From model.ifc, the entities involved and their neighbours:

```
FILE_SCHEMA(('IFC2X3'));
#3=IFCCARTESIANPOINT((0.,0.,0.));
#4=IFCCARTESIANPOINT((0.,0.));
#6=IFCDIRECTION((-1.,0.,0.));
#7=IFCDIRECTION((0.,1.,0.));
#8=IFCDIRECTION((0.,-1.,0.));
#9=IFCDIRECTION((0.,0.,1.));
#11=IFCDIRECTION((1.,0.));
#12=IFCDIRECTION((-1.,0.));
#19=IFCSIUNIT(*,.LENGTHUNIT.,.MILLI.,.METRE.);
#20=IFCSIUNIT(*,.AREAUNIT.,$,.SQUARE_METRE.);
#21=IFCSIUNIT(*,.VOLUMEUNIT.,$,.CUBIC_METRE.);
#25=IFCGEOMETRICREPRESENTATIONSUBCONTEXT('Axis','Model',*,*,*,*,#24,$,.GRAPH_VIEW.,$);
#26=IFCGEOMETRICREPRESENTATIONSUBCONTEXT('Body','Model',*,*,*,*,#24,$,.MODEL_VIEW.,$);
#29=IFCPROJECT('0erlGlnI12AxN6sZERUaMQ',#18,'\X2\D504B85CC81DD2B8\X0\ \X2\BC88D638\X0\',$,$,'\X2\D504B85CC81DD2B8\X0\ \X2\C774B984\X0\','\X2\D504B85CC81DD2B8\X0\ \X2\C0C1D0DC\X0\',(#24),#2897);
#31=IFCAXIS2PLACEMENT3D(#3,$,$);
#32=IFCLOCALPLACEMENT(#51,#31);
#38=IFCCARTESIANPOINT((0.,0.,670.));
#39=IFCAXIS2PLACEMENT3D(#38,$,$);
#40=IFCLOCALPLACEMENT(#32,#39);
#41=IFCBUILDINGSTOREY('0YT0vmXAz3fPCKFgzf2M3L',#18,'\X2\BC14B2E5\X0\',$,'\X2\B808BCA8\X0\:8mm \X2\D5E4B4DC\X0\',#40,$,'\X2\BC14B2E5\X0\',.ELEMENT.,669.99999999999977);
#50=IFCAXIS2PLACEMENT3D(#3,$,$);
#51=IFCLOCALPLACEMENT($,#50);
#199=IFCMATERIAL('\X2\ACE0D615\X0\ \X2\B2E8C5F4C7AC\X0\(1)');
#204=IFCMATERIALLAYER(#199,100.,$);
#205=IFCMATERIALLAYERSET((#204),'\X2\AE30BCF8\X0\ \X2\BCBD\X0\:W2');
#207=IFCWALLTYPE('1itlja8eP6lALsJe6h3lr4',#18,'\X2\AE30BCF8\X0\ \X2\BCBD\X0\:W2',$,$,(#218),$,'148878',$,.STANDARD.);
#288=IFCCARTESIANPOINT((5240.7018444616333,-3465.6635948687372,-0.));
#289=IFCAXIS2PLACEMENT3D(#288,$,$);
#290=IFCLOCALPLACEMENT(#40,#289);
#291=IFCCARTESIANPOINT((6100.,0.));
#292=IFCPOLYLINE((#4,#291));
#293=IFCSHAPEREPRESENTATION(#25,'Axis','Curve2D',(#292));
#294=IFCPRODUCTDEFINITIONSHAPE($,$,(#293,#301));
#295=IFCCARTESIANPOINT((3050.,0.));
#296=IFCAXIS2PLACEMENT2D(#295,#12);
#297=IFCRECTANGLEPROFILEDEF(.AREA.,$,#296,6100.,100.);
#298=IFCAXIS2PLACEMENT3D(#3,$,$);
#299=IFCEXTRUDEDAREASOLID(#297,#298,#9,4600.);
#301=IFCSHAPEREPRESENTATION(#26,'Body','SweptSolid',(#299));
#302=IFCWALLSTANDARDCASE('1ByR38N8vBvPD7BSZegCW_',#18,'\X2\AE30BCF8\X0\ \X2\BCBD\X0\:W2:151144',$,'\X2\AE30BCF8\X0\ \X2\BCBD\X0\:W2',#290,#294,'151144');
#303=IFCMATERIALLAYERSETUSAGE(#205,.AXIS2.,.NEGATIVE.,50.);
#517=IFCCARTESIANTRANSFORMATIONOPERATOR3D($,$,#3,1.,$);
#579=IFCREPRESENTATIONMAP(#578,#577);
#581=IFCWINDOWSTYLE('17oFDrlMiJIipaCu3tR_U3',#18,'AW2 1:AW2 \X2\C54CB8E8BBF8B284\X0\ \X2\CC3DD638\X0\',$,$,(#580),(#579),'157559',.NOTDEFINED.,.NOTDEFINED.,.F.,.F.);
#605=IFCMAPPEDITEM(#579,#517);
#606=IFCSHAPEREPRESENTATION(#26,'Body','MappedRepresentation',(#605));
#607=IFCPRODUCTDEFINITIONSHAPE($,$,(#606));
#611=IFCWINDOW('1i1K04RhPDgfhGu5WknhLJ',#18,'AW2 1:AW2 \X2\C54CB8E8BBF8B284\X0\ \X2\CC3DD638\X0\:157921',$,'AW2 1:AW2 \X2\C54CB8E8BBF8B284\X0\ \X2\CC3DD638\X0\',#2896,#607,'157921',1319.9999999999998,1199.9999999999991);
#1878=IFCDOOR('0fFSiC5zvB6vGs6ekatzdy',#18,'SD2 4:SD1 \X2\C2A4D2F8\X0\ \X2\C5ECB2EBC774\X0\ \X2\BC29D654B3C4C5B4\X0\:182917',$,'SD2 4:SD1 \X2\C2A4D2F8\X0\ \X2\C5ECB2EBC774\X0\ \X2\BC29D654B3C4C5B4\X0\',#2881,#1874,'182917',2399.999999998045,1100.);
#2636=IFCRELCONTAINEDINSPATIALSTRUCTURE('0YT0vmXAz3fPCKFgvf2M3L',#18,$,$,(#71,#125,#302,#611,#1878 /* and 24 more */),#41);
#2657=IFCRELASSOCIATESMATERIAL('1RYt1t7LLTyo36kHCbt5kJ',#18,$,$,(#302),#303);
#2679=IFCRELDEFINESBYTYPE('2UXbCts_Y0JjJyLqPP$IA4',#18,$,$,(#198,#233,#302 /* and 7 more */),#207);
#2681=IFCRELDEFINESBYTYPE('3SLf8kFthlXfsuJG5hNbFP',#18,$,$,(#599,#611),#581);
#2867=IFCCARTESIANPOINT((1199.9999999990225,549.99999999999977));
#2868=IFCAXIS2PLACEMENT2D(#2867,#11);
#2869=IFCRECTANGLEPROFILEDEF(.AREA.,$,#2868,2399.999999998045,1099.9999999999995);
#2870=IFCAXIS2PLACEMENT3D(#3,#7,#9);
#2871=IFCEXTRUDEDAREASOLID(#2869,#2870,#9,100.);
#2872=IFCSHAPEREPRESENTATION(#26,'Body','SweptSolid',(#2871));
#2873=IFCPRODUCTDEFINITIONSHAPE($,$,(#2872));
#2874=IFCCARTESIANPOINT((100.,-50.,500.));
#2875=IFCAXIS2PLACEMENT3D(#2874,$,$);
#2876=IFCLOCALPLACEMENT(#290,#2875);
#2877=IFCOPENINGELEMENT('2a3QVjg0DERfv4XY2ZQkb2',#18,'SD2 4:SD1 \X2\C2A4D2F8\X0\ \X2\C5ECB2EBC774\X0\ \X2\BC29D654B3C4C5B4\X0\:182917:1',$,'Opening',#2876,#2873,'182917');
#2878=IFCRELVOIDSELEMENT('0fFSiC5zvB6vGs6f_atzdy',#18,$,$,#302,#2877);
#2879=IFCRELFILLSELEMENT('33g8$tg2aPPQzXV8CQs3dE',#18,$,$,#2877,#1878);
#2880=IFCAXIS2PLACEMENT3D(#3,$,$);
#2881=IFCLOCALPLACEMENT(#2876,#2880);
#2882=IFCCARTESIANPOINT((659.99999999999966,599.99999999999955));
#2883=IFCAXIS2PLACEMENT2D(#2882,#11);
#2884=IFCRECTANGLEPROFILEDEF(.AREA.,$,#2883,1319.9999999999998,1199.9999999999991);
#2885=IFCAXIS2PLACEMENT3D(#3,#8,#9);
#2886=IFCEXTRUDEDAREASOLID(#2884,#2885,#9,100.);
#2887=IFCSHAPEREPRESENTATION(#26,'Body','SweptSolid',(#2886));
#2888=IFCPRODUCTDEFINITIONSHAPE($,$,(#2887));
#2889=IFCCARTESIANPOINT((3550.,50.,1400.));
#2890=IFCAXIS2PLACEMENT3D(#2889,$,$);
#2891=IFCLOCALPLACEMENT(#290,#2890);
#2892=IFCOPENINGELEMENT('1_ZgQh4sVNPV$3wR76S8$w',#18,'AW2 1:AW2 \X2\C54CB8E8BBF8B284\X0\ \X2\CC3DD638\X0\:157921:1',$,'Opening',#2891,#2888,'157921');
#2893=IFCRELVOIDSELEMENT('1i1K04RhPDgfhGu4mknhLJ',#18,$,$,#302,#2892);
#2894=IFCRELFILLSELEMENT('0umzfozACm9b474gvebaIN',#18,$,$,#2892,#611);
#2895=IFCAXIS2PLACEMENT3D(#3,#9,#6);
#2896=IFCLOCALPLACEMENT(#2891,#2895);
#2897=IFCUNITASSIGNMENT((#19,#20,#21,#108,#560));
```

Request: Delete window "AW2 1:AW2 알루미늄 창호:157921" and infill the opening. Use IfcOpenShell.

```python
import ifcopenshell
import ifcopenshell.api.feature
import ifcopenshell.api.root
import ifcopenshell.geom
import ifcopenshell.util.shape

model = ifcopenshell.open("model.ifc")
settings = ifcopenshell.geom.settings()


def volume(element):
    """Net volume in cubic metres, openings subtracted."""
    shape = ifcopenshell.geom.create_shape(settings, element)
    return ifcopenshell.util.shape.get_volume(shape.geometry)


window = model.by_guid("1i1K04RhPDgfhGu5WknhLJ")
opening = window.FillsVoids[0].RelatingOpeningElement
wall = opening.VoidsElements[0].RelatingBuildingElement
before = volume(wall)

ifcopenshell.api.root.remove_product(model, product=window)
ifcopenshell.api.feature.remove_feature(model, feature=opening)

after = volume(wall)

print(f"wall volume {before:.3f} -> {after:.3f} m3")

model.write("model_v2.ifc")
```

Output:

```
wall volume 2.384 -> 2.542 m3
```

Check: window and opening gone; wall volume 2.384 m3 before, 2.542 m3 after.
